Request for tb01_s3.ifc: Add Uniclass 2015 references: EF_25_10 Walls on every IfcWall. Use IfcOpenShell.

First a look at what the model holds.

```python
import ifcopenshell

model = ifcopenshell.open("tb01_s3.ifc")
print(model.schema)
print("classifications:", [c.Name for c in model.by_type("IfcClassification")])
for ifc_class in ("IfcDoor", "IfcRoof", "IfcStair", "IfcWall", "IfcWindow"):
    print(ifc_class, len(model.by_type(ifc_class)))
```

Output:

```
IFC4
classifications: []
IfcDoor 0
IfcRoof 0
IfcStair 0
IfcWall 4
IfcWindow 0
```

```python
import ifcopenshell
import ifcopenshell.api.classification

model = ifcopenshell.open("tb01_s3.ifc")

system = ifcopenshell.api.classification.add_classification(model, classification="Uniclass 2015")

codes = {
    "IfcWall": ("EF_25_10", "Walls"),
}
for ifc_class, (code, name) in codes.items():
    products = model.by_type(ifc_class)
    ifcopenshell.api.classification.add_reference(
        model, products=products, classification=system, identification=code, name=name
    )
    print(code, len(products))

model.write("tb01_s3-out.ifc")
```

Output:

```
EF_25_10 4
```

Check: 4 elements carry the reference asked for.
